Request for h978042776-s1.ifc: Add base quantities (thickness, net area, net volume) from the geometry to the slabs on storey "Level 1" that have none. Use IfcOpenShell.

First a look at what the model holds.

```python
import ifcopenshell
import ifcopenshell.util.element
import ifcopenshell.util.unit

model = ifcopenshell.open("h978042776-s1.ifc")
print(model.schema)
for unit_type in ("LENGTHUNIT", "AREAUNIT", "VOLUMEUNIT"):
    print(unit_type, ifcopenshell.util.unit.calculate_unit_scale(model, unit_type))
storey = next(s for s in model.by_type("IfcBuildingStorey") if s.Name == "Level 1")
slabs = [e for e in ifcopenshell.util.element.get_decomposition(storey) if e.is_a("IfcSlab")]
for e in sorted(slabs, key=lambda e: e.id()):
    print(e.id(), e.is_a(), e.Name, list(ifcopenshell.util.element.get_psets(e, qtos_only=True)), sep=" | ")
```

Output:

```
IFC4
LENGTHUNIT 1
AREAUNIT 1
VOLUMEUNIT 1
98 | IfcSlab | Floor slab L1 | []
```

```python
import ifcopenshell
import ifcopenshell.api.pset
import ifcopenshell.geom
import ifcopenshell.util.element
import ifcopenshell.util.shape
import ifcopenshell.util.unit

model = ifcopenshell.open("h978042776-s1.ifc")
unit_scale = ifcopenshell.util.unit.calculate_unit_scale(model)
area_scale = ifcopenshell.util.unit.calculate_unit_scale(model, "AREAUNIT")
volume_scale = ifcopenshell.util.unit.calculate_unit_scale(model, "VOLUMEUNIT")
settings = ifcopenshell.geom.settings()

storey = next(s for s in model.by_type("IfcBuildingStorey") if s.Name == "Level 1")
slabs = [e for e in ifcopenshell.util.element.get_decomposition(storey) if e.is_a("IfcSlab")]

for e in sorted(slabs, key=lambda e: e.id()):
    if ifcopenshell.util.element.get_psets(e, qtos_only=True, should_inherit=False):
        continue
    # Geometry comes back in metres, in the element's own axes.
    shape = ifcopenshell.geom.create_shape(settings, e)
    values = {
        "Width": ifcopenshell.util.shape.get_z(shape.geometry) / unit_scale,
        "NetArea": ifcopenshell.util.shape.get_footprint_area(shape.geometry) / area_scale,
        "NetVolume": ifcopenshell.util.shape.get_volume(shape.geometry) / volume_scale,
    }
    qto = ifcopenshell.api.pset.add_qto(model, product=e, name="Qto_SlabBaseQuantities")
    ifcopenshell.api.pset.edit_qto(model, qto=qto, properties=values)
    print(e.id(), {k: round(v, 3) for k, v in values.items()})

model.write("h978042776-s1_rev.ifc")
```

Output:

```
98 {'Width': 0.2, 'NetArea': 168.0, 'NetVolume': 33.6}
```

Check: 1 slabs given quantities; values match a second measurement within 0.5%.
